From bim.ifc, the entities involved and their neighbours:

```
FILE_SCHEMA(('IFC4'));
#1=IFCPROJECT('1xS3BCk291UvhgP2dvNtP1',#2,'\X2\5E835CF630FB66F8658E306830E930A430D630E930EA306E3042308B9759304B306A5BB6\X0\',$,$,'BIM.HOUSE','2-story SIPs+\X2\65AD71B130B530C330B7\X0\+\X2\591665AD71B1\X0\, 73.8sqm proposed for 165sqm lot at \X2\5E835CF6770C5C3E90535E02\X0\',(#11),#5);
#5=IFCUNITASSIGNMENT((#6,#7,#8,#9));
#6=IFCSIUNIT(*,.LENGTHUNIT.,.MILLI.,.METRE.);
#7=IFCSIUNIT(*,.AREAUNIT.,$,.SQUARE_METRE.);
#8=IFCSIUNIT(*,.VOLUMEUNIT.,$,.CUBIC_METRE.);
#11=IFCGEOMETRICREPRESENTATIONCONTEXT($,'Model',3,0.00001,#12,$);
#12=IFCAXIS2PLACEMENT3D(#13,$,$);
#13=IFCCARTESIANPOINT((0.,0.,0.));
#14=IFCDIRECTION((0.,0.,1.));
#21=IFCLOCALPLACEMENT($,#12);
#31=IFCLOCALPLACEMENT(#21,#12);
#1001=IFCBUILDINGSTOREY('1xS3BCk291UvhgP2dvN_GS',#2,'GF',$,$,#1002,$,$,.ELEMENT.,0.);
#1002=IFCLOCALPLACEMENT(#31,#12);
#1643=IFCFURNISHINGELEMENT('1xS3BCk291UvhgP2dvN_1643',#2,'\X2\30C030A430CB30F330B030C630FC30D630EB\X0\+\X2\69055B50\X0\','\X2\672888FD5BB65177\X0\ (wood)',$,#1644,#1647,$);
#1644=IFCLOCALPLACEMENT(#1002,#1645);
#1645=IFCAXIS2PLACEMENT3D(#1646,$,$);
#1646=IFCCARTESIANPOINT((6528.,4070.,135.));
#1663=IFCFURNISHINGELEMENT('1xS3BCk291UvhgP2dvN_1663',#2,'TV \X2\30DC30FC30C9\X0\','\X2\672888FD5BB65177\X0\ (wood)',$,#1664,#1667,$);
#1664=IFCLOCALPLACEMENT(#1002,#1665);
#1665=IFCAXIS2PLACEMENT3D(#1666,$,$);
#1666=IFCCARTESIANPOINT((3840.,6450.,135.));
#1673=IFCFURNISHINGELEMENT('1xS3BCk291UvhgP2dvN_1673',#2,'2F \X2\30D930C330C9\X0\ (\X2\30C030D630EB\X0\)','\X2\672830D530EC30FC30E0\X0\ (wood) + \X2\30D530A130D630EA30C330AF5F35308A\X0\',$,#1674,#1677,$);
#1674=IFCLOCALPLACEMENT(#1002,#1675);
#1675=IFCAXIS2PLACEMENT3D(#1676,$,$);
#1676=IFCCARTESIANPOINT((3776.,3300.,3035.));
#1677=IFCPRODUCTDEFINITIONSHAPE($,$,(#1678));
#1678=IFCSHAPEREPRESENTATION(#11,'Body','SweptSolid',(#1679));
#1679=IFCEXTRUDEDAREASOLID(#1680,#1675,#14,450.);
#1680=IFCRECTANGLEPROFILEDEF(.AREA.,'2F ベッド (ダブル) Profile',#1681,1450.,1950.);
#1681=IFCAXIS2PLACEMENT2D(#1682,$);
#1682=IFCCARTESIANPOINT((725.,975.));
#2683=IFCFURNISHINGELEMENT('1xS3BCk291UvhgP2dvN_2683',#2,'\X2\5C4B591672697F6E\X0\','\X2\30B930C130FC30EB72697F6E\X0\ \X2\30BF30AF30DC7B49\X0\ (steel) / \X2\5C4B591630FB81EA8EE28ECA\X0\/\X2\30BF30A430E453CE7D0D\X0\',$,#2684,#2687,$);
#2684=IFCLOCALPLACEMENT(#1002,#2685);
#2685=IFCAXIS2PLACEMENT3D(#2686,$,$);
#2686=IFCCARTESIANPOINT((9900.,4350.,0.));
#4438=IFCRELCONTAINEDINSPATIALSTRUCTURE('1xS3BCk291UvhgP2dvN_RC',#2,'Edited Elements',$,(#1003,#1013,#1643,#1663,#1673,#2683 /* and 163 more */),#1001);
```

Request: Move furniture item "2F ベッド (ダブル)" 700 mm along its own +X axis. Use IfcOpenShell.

```python
import ifcopenshell
import ifcopenshell.api.geometry
import ifcopenshell.util.placement

model = ifcopenshell.open("bim.ifc")

item = model.by_guid("1xS3BCk291UvhgP2dvN_1673")
matrix = ifcopenshell.util.placement.get_local_placement(item.ObjectPlacement)
matrix[:3, 3] += matrix[:3, 0] * 700.0
ifcopenshell.api.geometry.edit_object_placement(model, product=item, matrix=matrix, is_si=False)

print(ifcopenshell.util.placement.get_local_placement(item.ObjectPlacement).round(3) + 0.0)

model.write("bim_edited.ifc")
```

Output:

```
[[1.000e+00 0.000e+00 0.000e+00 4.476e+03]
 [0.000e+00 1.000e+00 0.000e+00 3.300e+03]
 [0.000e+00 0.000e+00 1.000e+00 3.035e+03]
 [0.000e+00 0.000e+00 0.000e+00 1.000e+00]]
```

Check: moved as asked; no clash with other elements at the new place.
